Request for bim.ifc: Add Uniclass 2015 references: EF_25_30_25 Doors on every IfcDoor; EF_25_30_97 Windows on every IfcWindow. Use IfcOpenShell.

First a look at what the model holds.

```python
import ifcopenshell

model = ifcopenshell.open("bim.ifc")
print(model.schema)
print("classifications:", [c.Name for c in model.by_type("IfcClassification")])
for ifc_class in ("IfcDoor", "IfcRoof", "IfcStair", "IfcWall", "IfcWindow"):
    print(ifc_class, len(model.by_type(ifc_class)))
```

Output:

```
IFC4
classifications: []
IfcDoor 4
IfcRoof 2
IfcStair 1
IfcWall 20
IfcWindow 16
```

```python
import ifcopenshell
import ifcopenshell.api.classification

model = ifcopenshell.open("bim.ifc")

system = ifcopenshell.api.classification.add_classification(model, classification="Uniclass 2015")

codes = {
    "IfcDoor": ("EF_25_30_25", "Doors"),
    "IfcWindow": ("EF_25_30_97", "Windows"),
}
for ifc_class, (code, name) in codes.items():
    products = model.by_type(ifc_class)
    ifcopenshell.api.classification.add_reference(
        model, products=products, classification=system, identification=code, name=name
    )
    print(code, len(products))

model.write("bim_edited.ifc")
```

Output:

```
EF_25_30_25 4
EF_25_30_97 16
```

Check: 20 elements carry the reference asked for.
